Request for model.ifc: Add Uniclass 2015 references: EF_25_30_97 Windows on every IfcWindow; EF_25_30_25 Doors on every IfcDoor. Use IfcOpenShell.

First a look at what the model holds.

```python
import ifcopenshell

model = ifcopenshell.open("model.ifc")
print(model.schema)
print("classifications:", [c.Name for c in model.by_type("IfcClassification")])
for ifc_class in ("IfcDoor", "IfcRoof", "IfcStair", "IfcWall", "IfcWindow"):
    print(ifc_class, len(model.by_type(ifc_class)))
```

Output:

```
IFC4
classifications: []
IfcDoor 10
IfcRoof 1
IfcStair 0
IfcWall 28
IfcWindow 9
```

```python
import ifcopenshell
import ifcopenshell.api.classification

model = ifcopenshell.open("model.ifc")

system = ifcopenshell.api.classification.add_classification(model, classification="Uniclass 2015")

codes = {
    "IfcWindow": ("EF_25_30_97", "Windows"),
    "IfcDoor": ("EF_25_30_25", "Doors"),
}
for ifc_class, (code, name) in codes.items():
    products = model.by_type(ifc_class)
    ifcopenshell.api.classification.add_reference(
        model, products=products, classification=system, identification=code, name=name
    )
    print(code, len(products))

model.write("model_rev.ifc")
```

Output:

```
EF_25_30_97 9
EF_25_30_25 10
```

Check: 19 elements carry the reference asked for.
